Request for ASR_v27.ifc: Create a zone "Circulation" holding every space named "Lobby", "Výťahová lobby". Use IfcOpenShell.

First a look at what the model holds.

```python
import ifcopenshell

model = ifcopenshell.open("ASR_v27.ifc")
print(model.schema)
seen = {}
for space in model.by_type("IfcSpace"):
    seen[space.LongName] = seen.get(space.LongName, 0) + 1
for name, count in sorted(seen.items(), key=str):
    print(count, "x", name)
print("zones:", [z.Name for z in model.by_type("IfcZone")][:20])
```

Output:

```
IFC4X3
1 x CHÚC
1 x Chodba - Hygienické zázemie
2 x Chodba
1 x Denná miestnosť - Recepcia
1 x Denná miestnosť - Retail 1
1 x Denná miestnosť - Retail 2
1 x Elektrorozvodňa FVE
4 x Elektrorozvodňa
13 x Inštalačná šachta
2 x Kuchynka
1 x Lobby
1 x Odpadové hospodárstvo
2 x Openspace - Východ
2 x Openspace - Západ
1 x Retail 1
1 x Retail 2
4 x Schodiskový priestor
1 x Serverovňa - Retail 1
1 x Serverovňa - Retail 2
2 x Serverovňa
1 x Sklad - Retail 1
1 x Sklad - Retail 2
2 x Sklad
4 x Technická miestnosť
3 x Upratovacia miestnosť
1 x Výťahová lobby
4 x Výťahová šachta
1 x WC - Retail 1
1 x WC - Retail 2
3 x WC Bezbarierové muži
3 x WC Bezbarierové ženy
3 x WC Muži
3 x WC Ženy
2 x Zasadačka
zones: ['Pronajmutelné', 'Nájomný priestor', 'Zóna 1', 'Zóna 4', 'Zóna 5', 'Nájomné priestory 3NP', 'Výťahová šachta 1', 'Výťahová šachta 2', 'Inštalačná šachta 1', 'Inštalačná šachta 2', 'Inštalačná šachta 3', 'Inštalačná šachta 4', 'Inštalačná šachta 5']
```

```python
import ifcopenshell
import ifcopenshell.api.group
import ifcopenshell.api.root

model = ifcopenshell.open("ASR_v27.ifc")

names = {"Lobby", "Výťahová lobby"}
spaces = [s for s in model.by_type("IfcSpace") if s.LongName in names]

zone = ifcopenshell.api.root.create_entity(model, ifc_class="IfcZone", name="Circulation")
ifcopenshell.api.group.assign_group(model, products=spaces, group=zone)
print(len(spaces), "spaces in", zone.Name)

model.write("ASR_v27_edited.ifc")
```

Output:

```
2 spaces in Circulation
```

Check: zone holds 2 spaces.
